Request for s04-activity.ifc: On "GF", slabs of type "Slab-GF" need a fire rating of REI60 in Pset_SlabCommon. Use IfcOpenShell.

First a look at what the model holds.

```python
import ifcopenshell
import ifcopenshell.util.element

model = ifcopenshell.open("s04-activity.ifc")
print(model.schema)
storey = next(s for s in model.by_type("IfcBuildingStorey") if s.Name == "GF")
slabs = [e for e in ifcopenshell.util.element.get_decomposition(storey) if e.is_a("IfcSlab")]
seen = {}
for e in slabs:
    element_type = ifcopenshell.util.element.get_type(e)
    key = (element_type.Name if element_type != e and element_type else None, ifcopenshell.util.element.get_pset(e, "Pset_SlabCommon", "FireRating"))
    seen[key] = seen.get(key, 0) + 1
for (name, value), count in sorted(seen.items(), key=str):
    print(count, "x", name, "|", value)
```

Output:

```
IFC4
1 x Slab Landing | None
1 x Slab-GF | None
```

```python
import ifcopenshell
import ifcopenshell.api.pset
import ifcopenshell.util.element

model = ifcopenshell.open("s04-activity.ifc")

storey = next(s for s in model.by_type("IfcBuildingStorey") if s.Name == "GF")
slabs = [e for e in ifcopenshell.util.element.get_decomposition(storey) if e.is_a("IfcSlab")]

count = 0
for e in slabs:
    element_type = ifcopenshell.util.element.get_type(e)
    if element_type in (None, e) or element_type.Name != "Slab-GF":
        continue
    # add_pset returns the element's existing set when there is one.
    pset = ifcopenshell.api.pset.add_pset(model, product=e, name="Pset_SlabCommon")
    ifcopenshell.api.pset.edit_pset(model, pset=pset, properties={"FireRating": "REI60"})
    count += 1

print(count, "slabs updated")

model.write("s04-activity_edited.ifc")
```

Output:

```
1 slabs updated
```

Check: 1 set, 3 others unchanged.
